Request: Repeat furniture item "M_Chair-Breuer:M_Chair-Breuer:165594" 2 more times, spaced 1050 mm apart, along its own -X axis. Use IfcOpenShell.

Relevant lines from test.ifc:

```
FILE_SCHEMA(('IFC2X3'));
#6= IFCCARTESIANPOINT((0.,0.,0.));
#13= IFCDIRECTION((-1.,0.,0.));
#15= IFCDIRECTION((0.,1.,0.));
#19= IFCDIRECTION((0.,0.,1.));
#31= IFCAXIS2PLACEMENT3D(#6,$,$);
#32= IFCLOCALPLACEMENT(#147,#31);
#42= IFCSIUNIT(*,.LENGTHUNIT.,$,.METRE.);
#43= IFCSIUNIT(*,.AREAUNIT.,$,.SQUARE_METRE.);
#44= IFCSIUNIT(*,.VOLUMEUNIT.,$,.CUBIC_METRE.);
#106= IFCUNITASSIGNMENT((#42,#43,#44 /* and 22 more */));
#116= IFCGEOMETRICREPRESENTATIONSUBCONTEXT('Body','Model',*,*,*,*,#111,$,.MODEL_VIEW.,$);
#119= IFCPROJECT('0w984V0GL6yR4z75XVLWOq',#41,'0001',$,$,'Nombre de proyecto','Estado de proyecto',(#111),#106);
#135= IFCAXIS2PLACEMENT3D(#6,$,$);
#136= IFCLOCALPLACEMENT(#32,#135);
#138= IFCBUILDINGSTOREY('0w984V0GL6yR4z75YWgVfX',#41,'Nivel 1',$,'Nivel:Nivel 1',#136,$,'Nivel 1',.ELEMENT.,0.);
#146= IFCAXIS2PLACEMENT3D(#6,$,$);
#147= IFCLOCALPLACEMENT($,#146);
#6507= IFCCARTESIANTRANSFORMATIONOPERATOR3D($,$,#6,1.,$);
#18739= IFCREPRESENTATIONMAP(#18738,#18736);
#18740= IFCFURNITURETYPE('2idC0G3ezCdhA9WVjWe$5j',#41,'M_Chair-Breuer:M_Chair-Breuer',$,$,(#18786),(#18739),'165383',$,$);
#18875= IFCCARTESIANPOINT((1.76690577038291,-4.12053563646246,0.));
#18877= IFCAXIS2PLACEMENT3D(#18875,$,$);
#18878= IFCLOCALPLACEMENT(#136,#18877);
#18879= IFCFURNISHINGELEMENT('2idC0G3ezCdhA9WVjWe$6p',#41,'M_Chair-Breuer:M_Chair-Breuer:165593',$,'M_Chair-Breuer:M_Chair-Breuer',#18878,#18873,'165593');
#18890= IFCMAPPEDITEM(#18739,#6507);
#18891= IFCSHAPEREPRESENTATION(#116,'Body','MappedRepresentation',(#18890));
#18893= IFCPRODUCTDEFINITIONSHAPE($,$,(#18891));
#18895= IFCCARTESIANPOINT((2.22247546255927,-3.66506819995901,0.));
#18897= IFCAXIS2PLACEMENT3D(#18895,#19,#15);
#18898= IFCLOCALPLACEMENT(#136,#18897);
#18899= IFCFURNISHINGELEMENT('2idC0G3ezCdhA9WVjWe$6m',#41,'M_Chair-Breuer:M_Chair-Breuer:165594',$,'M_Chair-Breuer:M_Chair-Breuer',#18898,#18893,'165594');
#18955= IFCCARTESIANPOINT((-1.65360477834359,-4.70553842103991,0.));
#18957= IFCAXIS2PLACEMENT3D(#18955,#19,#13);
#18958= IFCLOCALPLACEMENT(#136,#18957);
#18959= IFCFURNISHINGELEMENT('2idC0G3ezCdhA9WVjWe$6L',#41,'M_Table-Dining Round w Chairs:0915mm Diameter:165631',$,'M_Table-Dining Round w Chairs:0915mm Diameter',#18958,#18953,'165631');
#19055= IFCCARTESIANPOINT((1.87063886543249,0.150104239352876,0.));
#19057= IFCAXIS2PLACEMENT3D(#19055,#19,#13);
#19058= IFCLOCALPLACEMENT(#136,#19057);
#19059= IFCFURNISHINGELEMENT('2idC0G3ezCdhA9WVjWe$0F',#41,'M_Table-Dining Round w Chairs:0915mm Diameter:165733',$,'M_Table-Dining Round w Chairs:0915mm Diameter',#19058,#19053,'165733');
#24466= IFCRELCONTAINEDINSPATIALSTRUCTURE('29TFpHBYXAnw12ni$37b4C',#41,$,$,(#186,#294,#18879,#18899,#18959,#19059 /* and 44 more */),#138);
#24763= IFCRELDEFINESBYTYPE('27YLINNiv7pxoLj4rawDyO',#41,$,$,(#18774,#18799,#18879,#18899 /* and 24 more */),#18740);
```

```python
import ifcopenshell
import ifcopenshell.api.geometry
import ifcopenshell.api.root
import ifcopenshell.util.element
import ifcopenshell.util.placement
import ifcopenshell.util.unit

model = ifcopenshell.open("test.ifc")
unit_scale = ifcopenshell.util.unit.calculate_unit_scale(model)


def reuse_history(source, copy):
    """copy_class also copies each property set's owner history, people and application; keep the originals."""
    for rel in copy.IsDefinedBy:
        if rel.is_a("IfcRelDefinesByProperties") and (history := rel.RelatingPropertyDefinition.OwnerHistory):
            rel.RelatingPropertyDefinition.OwnerHistory = source.OwnerHistory
            ifcopenshell.util.element.remove_deep2(model, history)


source = model.by_id(18899)
base = ifcopenshell.util.placement.get_local_placement(source.ObjectPlacement)
step = -base[:3, 0] * 1.05 / unit_scale

for i in range(1, 3):
    copy = ifcopenshell.api.root.copy_class(model, product=source)
    copy.Representation = ifcopenshell.util.element.copy_deep(
        model, source.Representation, exclude=["IfcGeometricRepresentationContext", "IfcRepresentationMap"]
    )
    copy.Name = "M_Chair-Breuer:M_Chair-Breuer"
    copy.Tag = None
    reuse_history(source, copy)
    matrix = base.copy()
    matrix[:3, 3] += i * step
    print("added at", matrix[:3, 3].round(3) + 0.0)
    ifcopenshell.api.geometry.edit_object_placement(model, product=copy, matrix=matrix, is_si=False)

model.write("test_rev.ifc")
```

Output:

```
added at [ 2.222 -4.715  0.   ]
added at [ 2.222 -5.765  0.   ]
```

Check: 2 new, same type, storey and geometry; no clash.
